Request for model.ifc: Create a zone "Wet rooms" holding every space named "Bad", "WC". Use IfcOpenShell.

First a look at what the model holds.

```python
import ifcopenshell

model = ifcopenshell.open("model.ifc")
print(model.schema)
seen = {}
for space in model.by_type("IfcSpace"):
    seen[space.LongName] = seen.get(space.LongName, 0) + 1
for name, count in sorted(seen.items(), key=str):
    print(count, "x", name)
print("zones:", [z.Name for z in model.by_type("IfcZone")][:20])
```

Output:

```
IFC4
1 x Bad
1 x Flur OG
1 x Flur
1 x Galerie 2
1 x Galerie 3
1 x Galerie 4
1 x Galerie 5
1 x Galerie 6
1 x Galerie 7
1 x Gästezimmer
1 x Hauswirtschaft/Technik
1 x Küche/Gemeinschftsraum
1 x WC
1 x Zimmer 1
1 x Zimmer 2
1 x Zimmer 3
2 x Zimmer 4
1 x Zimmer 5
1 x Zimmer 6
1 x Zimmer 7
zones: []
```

```python
import ifcopenshell
import ifcopenshell.api.group
import ifcopenshell.api.root

model = ifcopenshell.open("model.ifc")

names = {"Bad", "WC"}
spaces = [s for s in model.by_type("IfcSpace") if s.LongName in names]

zone = ifcopenshell.api.root.create_entity(model, ifc_class="IfcZone", name="Wet rooms")
ifcopenshell.api.group.assign_group(model, products=spaces, group=zone)
print(len(spaces), "spaces in", zone.Name)

model.write("model_rev.ifc")
```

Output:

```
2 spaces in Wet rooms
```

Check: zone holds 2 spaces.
